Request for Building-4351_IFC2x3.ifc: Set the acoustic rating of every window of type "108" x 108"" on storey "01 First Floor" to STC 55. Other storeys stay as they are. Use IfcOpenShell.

First a look at what the model holds.

```python
import ifcopenshell
import ifcopenshell.util.element

model = ifcopenshell.open("Building-4351_IFC2x3.ifc")
print(model.schema)
storey = next(s for s in model.by_type("IfcBuildingStorey") if s.Name == "01 First Floor")
windows = [e for e in ifcopenshell.util.element.get_decomposition(storey) if e.is_a("IfcWindow")]
seen = {}
for e in windows:
    element_type = ifcopenshell.util.element.get_type(e)
    key = (element_type.Name if element_type != e and element_type else None, ifcopenshell.util.element.get_pset(e, "Pset_WindowCommon", "AcousticRating"))
    seen[key] = seen.get(key, 0) + 1
for (name, value), count in sorted(seen.items(), key=str):
    print(count, "x", name, "|", value)
```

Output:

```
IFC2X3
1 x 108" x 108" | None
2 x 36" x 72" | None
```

```python
import ifcopenshell
import ifcopenshell.api.pset
import ifcopenshell.util.element

model = ifcopenshell.open("Building-4351_IFC2x3.ifc")

storey = next(s for s in model.by_type("IfcBuildingStorey") if s.Name == "01 First Floor")
windows = [e for e in ifcopenshell.util.element.get_decomposition(storey) if e.is_a("IfcWindow")]

count = 0
for e in windows:
    element_type = ifcopenshell.util.element.get_type(e)
    if element_type in (None, e) or element_type.Name != '108" x 108"':
        continue
    # add_pset returns the element's existing set when there is one.
    pset = ifcopenshell.api.pset.add_pset(model, product=e, name="Pset_WindowCommon")
    ifcopenshell.api.pset.edit_pset(model, pset=pset, properties={"AcousticRating": "STC 55"})
    count += 1

print(count, "windows updated")

model.write("Building-4351_IFC2x3_rev.ifc")
```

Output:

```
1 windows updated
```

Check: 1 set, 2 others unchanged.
